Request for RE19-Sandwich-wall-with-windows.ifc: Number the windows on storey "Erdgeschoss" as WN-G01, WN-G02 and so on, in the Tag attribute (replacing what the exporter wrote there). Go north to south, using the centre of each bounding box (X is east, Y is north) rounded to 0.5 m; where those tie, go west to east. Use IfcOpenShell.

First a look at what the model holds.

```python
import ifcopenshell
import ifcopenshell.util.element
import ifcopenshell.util.placement

model = ifcopenshell.open("RE19-Sandwich-wall-with-windows.ifc")
print(model.schema)
storey = next(s for s in model.by_type("IfcBuildingStorey") if s.Name == "Erdgeschoss")
windows = [e for e in ifcopenshell.util.element.get_decomposition(storey) if e.is_a("IfcWindow")]
for e in sorted(windows, key=lambda e: e.id()):
    origin = ifcopenshell.util.placement.get_local_placement(e.ObjectPlacement)[:3, 3]
    print(e.id(), e.Tag, e.Name, origin.round(2) + 0.0, sep=" | ")
```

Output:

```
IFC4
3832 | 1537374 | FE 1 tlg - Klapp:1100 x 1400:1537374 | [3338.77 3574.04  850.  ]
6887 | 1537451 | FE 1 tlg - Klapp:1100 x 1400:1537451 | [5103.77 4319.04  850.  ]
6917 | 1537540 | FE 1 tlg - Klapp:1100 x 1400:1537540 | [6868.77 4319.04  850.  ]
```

```python
import ifcopenshell
import ifcopenshell.geom
import ifcopenshell.util.element
import ifcopenshell.util.shape

model = ifcopenshell.open("RE19-Sandwich-wall-with-windows.ifc")
settings = ifcopenshell.geom.settings()
settings.set("use-world-coords", True)


def centre(element):
    shape = ifcopenshell.geom.create_shape(settings, element)
    return ifcopenshell.util.shape.get_bbox_centroid(shape.geometry)


storey = next(s for s in model.by_type("IfcBuildingStorey") if s.Name == "Erdgeschoss")
windows = [e for e in ifcopenshell.util.element.get_decomposition(storey) if e.is_a("IfcWindow")]

# Insertion points can sit at a corner or the storey origin, so sort by the geometry (in metres).
centres = {e: centre(e) for e in windows}
windows.sort(key=lambda e: (-round(centres[e][1] / 0.5), centres[e][0]))

for i, e in enumerate(windows, start=1):
    number = f"WN-G{i:02d}"
    e.Tag = number
    print(e.id(), number)

model.write("RE19-Sandwich-wall-with-windows-out.ifc")
```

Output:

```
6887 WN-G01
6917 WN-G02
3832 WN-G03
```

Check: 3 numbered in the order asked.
